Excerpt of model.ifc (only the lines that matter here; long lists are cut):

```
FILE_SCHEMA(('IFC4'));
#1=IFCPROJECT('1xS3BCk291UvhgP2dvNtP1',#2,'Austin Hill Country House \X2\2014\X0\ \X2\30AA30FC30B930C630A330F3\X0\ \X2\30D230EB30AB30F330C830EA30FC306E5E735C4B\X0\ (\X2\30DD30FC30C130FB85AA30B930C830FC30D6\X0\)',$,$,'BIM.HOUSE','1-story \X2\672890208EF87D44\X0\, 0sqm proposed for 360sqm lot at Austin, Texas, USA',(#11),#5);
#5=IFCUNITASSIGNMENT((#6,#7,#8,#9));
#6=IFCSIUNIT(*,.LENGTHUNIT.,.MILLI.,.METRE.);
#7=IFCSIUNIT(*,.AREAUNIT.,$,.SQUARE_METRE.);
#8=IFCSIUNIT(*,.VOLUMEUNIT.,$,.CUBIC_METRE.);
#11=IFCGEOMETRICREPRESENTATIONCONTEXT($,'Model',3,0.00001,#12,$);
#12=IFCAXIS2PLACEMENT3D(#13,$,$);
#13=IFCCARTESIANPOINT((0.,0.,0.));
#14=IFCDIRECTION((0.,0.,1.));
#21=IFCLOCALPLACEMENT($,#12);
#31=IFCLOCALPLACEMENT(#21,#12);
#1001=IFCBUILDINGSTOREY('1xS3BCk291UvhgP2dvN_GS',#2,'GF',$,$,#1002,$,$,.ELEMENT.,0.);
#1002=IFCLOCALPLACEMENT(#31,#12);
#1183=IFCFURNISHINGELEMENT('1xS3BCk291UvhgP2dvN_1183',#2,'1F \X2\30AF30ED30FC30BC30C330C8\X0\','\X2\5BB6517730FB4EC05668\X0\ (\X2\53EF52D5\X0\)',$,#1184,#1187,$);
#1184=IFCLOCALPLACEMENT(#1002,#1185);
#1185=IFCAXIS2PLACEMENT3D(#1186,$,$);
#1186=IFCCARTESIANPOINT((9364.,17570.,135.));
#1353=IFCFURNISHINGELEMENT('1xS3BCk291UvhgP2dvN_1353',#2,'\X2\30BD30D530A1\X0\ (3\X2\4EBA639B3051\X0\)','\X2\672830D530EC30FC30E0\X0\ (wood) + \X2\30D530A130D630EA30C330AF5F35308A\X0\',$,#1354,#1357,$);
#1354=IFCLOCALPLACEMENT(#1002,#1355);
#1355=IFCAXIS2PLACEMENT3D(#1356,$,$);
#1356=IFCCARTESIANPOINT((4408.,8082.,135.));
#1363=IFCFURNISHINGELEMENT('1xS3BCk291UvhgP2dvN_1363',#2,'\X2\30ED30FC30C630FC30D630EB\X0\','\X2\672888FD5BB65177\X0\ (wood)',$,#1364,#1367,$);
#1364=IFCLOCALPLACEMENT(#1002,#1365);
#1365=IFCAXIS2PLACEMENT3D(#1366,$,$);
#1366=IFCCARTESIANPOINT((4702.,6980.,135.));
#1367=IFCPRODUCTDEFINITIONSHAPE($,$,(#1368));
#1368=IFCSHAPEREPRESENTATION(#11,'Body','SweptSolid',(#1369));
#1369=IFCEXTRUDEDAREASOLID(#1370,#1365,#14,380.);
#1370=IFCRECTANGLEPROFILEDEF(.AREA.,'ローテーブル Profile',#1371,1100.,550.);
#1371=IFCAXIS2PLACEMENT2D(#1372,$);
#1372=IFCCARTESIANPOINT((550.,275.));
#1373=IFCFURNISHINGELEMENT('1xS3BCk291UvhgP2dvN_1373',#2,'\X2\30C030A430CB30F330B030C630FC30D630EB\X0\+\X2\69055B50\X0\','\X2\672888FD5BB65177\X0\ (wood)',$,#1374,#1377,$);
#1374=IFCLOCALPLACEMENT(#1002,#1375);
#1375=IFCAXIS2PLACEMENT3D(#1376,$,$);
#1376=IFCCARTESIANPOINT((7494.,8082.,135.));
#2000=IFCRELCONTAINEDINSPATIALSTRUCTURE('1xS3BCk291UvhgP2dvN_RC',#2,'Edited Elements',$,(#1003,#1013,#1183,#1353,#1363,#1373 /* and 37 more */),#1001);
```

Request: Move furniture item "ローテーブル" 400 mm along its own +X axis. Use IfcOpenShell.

```python
import ifcopenshell
import ifcopenshell.api.geometry
import ifcopenshell.util.placement
import ifcopenshell.util.unit

model = ifcopenshell.open("model.ifc")
unit_scale = ifcopenshell.util.unit.calculate_unit_scale(model)

item = model.by_guid("1xS3BCk291UvhgP2dvN_1363")
matrix = ifcopenshell.util.placement.get_local_placement(item.ObjectPlacement)
matrix[:3, 3] += matrix[:3, 0] * 0.4 / unit_scale
ifcopenshell.api.geometry.edit_object_placement(model, product=item, matrix=matrix, is_si=False)

print(ifcopenshell.util.placement.get_local_placement(item.ObjectPlacement).round(3) + 0.0)

model.write("model-out.ifc")
```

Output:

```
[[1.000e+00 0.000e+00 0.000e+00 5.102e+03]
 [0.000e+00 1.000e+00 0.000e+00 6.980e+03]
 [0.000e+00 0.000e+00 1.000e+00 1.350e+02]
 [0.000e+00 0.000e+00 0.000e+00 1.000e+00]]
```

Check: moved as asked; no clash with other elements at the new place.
